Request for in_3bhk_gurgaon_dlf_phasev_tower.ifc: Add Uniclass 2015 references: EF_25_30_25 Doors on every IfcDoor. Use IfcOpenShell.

First a look at what the model holds.

```python
import ifcopenshell

model = ifcopenshell.open("in_3bhk_gurgaon_dlf_phasev_tower.ifc")
print(model.schema)
print("classifications:", [c.Name for c in model.by_type("IfcClassification")])
for ifc_class in ("IfcDoor", "IfcRoof", "IfcStair", "IfcWall", "IfcWindow"):
    print(ifc_class, len(model.by_type(ifc_class)))
```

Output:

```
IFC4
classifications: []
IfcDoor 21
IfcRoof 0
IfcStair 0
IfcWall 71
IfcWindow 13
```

```python
import ifcopenshell
import ifcopenshell.api.classification

model = ifcopenshell.open("in_3bhk_gurgaon_dlf_phasev_tower.ifc")

system = ifcopenshell.api.classification.add_classification(model, classification="Uniclass 2015")

codes = {
    "IfcDoor": ("EF_25_30_25", "Doors"),
}
for ifc_class, (code, name) in codes.items():
    products = model.by_type(ifc_class)
    ifcopenshell.api.classification.add_reference(
        model, products=products, classification=system, identification=code, name=name
    )
    print(code, len(products))

model.write("in_3bhk_gurgaon_dlf_phasev_tower-out.ifc")
```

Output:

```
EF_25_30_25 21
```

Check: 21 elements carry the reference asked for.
